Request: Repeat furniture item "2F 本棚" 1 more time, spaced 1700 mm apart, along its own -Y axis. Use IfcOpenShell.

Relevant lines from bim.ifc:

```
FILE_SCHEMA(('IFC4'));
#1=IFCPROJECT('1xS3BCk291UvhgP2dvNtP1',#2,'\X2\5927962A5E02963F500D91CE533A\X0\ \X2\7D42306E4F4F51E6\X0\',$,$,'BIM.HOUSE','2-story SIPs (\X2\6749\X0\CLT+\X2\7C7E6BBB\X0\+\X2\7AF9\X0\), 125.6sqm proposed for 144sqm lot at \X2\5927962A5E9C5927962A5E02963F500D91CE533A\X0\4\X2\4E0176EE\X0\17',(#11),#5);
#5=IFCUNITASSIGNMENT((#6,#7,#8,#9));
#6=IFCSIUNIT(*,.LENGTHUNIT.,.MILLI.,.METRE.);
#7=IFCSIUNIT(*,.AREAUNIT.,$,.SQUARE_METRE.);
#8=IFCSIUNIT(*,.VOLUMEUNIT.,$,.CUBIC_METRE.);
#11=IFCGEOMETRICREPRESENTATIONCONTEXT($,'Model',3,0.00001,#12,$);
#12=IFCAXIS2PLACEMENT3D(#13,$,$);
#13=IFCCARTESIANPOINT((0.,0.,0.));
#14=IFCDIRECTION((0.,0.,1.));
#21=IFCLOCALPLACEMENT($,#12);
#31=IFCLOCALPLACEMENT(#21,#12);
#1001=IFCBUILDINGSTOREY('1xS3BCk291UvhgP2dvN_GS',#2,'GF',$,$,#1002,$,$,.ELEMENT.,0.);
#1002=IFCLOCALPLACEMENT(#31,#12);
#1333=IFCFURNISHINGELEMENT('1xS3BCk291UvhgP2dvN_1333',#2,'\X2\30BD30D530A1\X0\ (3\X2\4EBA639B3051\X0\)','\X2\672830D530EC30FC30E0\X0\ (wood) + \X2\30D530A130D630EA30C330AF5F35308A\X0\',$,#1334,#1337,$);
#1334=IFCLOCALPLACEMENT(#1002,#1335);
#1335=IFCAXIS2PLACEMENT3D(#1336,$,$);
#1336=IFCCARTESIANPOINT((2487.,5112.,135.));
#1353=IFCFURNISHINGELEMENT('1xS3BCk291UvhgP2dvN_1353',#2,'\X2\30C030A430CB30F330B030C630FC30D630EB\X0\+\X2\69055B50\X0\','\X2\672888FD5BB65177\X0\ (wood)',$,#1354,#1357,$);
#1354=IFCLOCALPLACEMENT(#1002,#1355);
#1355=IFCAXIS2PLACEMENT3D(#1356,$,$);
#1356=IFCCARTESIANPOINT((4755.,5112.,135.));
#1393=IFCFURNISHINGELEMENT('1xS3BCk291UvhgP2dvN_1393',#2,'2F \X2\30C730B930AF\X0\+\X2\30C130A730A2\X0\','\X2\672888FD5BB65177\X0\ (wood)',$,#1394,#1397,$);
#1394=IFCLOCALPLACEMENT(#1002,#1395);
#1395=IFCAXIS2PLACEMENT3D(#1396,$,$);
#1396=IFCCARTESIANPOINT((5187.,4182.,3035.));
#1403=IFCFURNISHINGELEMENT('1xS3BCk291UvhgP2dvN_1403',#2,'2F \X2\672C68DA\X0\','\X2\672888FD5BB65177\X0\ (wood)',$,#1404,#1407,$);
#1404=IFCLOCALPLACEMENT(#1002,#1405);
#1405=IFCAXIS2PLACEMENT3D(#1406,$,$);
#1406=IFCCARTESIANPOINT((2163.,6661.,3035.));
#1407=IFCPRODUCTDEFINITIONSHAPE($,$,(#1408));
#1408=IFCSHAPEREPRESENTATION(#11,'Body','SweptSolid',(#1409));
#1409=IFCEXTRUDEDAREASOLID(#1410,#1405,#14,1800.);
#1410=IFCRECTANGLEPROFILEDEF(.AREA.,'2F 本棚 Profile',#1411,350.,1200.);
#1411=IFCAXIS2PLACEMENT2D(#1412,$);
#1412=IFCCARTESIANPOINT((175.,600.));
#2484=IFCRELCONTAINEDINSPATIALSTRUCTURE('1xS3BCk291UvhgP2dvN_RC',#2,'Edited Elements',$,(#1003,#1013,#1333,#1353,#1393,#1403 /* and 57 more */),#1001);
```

```python
import ifcopenshell
import ifcopenshell.api.geometry
import ifcopenshell.api.root
import ifcopenshell.util.element
import ifcopenshell.util.placement
import ifcopenshell.util.unit

model = ifcopenshell.open("bim.ifc")
unit_scale = ifcopenshell.util.unit.calculate_unit_scale(model)


def reuse_history(source, copy):
    """copy_class also copies each property set's owner history, people and application; keep the originals."""
    for rel in copy.IsDefinedBy:
        if rel.is_a("IfcRelDefinesByProperties") and (history := rel.RelatingPropertyDefinition.OwnerHistory):
            rel.RelatingPropertyDefinition.OwnerHistory = source.OwnerHistory
            ifcopenshell.util.element.remove_deep2(model, history)


source = model.by_guid("1xS3BCk291UvhgP2dvN_1403")
base = ifcopenshell.util.placement.get_local_placement(source.ObjectPlacement)
step = -base[:3, 1] * 1.7 / unit_scale

for i in range(1, 2):
    copy = ifcopenshell.api.root.copy_class(model, product=source)
    copy.Representation = ifcopenshell.util.element.copy_deep(
        model, source.Representation, exclude=["IfcGeometricRepresentationContext", "IfcRepresentationMap"]
    )
    reuse_history(source, copy)
    matrix = base.copy()
    matrix[:3, 3] += i * step
    print("added at", matrix[:3, 3].round(3) + 0.0)
    ifcopenshell.api.geometry.edit_object_placement(model, product=copy, matrix=matrix, is_si=False)

model.write("bim_rev.ifc")
```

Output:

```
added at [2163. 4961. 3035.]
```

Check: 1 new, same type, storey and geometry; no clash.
